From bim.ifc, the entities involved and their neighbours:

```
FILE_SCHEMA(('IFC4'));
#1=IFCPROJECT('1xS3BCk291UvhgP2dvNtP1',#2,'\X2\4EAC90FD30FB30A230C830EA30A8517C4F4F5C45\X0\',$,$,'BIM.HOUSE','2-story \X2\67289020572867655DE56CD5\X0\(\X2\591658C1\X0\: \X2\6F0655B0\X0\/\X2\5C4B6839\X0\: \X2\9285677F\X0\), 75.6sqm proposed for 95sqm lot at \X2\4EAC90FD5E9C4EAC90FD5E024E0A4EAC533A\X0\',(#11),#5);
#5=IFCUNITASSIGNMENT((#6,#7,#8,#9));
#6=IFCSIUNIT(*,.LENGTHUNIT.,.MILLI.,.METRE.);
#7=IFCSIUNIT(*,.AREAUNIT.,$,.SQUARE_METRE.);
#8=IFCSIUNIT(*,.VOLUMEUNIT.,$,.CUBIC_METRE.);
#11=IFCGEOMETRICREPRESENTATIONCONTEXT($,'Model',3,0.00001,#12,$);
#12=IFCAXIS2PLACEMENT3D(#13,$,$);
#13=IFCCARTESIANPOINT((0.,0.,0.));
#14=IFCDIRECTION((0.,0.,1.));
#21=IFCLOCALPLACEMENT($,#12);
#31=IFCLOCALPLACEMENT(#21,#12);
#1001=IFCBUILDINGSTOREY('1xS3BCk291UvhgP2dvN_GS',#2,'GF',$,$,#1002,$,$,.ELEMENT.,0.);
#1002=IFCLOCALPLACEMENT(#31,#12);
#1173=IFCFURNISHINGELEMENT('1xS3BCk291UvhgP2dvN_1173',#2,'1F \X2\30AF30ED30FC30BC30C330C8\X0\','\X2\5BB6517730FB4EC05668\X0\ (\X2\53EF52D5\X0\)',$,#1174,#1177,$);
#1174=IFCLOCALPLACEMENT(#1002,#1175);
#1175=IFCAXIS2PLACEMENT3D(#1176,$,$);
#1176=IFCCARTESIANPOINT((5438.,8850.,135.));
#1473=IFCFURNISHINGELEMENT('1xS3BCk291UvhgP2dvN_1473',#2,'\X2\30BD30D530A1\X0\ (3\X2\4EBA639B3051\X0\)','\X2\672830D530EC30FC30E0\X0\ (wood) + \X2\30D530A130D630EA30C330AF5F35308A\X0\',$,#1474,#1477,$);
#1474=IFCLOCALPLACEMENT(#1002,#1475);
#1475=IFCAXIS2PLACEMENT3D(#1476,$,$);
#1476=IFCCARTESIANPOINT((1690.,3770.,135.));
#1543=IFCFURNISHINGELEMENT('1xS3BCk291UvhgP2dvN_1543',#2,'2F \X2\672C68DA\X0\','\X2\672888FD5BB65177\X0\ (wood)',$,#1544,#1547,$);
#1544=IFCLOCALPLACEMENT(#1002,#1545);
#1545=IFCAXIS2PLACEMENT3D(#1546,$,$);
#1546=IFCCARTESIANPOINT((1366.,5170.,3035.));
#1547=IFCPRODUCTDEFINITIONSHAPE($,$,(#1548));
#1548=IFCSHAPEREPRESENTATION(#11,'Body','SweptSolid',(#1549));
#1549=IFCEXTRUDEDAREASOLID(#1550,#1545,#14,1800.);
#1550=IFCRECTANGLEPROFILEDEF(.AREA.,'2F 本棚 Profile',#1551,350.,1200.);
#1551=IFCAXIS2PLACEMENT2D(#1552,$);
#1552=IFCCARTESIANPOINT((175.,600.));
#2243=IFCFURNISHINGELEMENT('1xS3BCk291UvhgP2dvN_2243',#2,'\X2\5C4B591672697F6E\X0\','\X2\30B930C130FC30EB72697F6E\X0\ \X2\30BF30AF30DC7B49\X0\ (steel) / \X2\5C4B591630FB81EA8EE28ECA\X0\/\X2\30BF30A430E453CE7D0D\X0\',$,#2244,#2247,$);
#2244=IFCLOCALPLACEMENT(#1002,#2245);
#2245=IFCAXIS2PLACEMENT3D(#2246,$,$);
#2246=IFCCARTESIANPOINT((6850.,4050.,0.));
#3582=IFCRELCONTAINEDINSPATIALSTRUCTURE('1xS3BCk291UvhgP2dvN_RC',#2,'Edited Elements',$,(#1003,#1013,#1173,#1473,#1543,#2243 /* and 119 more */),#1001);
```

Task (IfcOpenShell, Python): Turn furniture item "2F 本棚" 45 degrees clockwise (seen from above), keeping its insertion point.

```python
import ifcopenshell
import ifcopenshell.api.geometry
import ifcopenshell.util.placement

model = ifcopenshell.open("bim.ifc")

item = model.by_guid("1xS3BCk291UvhgP2dvN_1543")
matrix = ifcopenshell.util.placement.get_local_placement(item.ObjectPlacement)
matrix = matrix @ ifcopenshell.util.placement.rotation(-45, "Z")
ifcopenshell.api.geometry.edit_object_placement(model, product=item, matrix=matrix, is_si=False)

print(ifcopenshell.util.placement.get_local_placement(item.ObjectPlacement).round(3) + 0.0)

model.write("bim_rev.ifc")
```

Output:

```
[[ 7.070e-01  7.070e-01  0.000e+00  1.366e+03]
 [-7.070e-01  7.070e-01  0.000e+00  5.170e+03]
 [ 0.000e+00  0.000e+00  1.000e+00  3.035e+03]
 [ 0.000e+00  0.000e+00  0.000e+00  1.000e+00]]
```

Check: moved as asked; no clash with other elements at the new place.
